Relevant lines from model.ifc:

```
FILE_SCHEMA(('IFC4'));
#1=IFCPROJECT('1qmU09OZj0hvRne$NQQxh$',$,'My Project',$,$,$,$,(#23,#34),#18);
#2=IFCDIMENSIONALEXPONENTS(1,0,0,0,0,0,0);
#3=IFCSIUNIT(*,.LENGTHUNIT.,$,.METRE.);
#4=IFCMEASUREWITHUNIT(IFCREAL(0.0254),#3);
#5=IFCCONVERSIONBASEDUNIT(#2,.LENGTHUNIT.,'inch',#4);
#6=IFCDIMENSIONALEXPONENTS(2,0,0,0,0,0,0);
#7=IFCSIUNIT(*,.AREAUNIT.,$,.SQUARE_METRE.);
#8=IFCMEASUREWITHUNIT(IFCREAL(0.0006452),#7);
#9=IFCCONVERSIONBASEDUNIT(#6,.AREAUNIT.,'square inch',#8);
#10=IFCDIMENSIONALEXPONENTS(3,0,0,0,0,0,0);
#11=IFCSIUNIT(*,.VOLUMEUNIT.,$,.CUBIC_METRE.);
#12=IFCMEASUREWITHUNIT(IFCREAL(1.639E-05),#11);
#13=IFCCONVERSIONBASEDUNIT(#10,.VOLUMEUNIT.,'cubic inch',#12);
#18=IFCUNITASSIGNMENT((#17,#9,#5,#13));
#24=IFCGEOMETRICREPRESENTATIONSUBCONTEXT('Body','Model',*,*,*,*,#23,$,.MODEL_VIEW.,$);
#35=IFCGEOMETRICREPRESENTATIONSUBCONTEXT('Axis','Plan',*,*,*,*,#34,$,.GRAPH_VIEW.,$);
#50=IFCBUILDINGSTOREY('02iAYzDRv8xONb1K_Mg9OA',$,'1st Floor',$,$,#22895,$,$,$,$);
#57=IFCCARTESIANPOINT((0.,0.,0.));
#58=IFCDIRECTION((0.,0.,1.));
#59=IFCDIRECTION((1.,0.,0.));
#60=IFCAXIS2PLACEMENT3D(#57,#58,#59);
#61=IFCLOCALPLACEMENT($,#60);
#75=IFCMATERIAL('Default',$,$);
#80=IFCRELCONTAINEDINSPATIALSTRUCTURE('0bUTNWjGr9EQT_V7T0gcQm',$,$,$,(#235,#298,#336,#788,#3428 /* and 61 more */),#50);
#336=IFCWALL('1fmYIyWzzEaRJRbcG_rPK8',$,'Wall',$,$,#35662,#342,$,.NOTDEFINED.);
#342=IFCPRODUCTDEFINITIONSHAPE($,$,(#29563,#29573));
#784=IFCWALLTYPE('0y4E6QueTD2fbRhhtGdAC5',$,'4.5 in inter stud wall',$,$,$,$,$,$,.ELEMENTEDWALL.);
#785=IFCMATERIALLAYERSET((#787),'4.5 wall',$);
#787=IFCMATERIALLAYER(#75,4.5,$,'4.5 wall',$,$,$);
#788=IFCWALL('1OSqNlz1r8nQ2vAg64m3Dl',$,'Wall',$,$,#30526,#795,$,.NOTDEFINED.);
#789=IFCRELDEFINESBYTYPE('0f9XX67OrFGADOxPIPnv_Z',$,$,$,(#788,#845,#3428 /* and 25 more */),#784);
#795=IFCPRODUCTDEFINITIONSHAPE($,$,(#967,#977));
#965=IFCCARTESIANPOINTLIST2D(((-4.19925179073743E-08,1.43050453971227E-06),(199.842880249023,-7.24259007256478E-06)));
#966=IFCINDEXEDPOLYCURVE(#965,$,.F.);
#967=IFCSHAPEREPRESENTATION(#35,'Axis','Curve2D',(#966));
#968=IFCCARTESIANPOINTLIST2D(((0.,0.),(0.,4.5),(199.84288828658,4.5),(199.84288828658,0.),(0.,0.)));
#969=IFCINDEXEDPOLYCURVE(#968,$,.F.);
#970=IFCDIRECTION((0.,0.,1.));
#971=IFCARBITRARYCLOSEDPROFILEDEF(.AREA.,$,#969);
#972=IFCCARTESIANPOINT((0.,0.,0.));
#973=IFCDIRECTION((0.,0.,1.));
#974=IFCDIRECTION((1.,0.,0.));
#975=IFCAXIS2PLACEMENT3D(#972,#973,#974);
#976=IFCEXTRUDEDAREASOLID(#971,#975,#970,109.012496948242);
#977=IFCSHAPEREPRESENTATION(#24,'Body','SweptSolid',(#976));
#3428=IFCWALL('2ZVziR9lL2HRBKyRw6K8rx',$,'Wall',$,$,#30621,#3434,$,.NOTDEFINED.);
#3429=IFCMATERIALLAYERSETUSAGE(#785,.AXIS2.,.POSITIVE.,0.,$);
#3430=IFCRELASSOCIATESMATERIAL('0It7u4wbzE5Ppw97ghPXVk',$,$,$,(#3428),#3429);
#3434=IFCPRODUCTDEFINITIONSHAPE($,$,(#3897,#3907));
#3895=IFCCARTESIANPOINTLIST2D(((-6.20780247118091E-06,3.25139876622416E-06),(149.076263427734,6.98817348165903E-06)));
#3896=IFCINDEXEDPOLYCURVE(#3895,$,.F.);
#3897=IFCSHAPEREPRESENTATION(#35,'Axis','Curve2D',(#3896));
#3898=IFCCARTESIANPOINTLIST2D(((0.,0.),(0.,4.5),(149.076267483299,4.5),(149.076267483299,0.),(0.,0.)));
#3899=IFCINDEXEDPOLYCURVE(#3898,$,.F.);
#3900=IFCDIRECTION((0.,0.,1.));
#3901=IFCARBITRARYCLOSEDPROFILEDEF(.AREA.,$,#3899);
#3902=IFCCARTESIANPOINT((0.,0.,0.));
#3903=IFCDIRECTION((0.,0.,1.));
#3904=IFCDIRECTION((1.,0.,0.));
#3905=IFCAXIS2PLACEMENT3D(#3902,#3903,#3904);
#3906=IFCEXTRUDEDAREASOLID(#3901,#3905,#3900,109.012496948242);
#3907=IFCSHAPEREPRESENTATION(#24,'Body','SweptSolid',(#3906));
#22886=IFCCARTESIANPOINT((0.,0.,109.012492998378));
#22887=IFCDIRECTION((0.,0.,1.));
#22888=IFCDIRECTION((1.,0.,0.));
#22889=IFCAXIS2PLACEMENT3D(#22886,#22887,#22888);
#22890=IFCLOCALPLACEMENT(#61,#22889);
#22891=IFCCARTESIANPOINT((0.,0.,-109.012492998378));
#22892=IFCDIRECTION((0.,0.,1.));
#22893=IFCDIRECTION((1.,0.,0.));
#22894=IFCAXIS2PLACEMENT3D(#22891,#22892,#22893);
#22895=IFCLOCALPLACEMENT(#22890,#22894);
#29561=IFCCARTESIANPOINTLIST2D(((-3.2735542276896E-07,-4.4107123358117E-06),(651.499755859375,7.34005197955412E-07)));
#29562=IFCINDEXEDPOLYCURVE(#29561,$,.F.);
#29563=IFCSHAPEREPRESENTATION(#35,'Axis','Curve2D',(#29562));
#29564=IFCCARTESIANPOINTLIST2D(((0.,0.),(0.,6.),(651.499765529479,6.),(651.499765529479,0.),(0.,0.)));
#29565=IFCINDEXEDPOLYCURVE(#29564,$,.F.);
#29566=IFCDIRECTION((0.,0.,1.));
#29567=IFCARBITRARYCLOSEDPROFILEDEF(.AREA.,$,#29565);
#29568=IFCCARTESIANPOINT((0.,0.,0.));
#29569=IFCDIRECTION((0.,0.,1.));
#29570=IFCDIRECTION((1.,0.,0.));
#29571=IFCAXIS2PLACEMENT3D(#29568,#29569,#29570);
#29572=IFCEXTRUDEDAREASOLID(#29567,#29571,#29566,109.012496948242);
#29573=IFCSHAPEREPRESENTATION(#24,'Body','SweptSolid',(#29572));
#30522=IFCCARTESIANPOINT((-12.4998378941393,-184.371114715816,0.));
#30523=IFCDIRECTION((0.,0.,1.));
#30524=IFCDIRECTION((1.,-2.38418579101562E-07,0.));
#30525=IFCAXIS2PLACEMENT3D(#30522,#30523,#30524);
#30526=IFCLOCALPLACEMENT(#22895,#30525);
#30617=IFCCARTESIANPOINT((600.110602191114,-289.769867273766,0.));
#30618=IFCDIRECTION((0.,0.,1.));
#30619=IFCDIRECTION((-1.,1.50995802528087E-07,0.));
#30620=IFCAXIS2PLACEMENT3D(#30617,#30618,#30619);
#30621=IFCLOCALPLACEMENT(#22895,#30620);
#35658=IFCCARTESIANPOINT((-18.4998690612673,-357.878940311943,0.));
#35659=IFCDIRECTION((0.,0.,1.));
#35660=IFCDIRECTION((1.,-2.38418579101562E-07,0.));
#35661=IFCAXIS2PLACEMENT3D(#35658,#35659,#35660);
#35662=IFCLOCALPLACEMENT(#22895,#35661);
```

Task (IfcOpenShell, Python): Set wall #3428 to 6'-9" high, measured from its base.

```python
import ifcopenshell
import ifcopenshell.geom
import ifcopenshell.util.representation
import ifcopenshell.util.shape
import ifcopenshell.util.unit

model = ifcopenshell.open("model.ifc")
unit_scale = ifcopenshell.util.unit.calculate_unit_scale(model)
settings = ifcopenshell.geom.settings()


def volume(element):
    """Net volume in cubic metres, openings subtracted."""
    shape = ifcopenshell.geom.create_shape(settings, element)
    return ifcopenshell.util.shape.get_volume(shape.geometry)


wall = model.by_id(3428)
before = volume(wall)

body = ifcopenshell.util.representation.get_representation(wall, "Model", "Body")
solid = body.Items[0]
old_height = solid.Depth
solid.Depth = 81 * 0.0254 / unit_scale
after = volume(wall)

print(f"height {old_height:g} -> {solid.Depth:g}, volume {before:.3f} -> {after:.3f} m3")

model.write("model_rev.ifc")
```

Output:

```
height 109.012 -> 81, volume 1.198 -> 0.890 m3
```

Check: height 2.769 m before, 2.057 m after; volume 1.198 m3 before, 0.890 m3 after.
